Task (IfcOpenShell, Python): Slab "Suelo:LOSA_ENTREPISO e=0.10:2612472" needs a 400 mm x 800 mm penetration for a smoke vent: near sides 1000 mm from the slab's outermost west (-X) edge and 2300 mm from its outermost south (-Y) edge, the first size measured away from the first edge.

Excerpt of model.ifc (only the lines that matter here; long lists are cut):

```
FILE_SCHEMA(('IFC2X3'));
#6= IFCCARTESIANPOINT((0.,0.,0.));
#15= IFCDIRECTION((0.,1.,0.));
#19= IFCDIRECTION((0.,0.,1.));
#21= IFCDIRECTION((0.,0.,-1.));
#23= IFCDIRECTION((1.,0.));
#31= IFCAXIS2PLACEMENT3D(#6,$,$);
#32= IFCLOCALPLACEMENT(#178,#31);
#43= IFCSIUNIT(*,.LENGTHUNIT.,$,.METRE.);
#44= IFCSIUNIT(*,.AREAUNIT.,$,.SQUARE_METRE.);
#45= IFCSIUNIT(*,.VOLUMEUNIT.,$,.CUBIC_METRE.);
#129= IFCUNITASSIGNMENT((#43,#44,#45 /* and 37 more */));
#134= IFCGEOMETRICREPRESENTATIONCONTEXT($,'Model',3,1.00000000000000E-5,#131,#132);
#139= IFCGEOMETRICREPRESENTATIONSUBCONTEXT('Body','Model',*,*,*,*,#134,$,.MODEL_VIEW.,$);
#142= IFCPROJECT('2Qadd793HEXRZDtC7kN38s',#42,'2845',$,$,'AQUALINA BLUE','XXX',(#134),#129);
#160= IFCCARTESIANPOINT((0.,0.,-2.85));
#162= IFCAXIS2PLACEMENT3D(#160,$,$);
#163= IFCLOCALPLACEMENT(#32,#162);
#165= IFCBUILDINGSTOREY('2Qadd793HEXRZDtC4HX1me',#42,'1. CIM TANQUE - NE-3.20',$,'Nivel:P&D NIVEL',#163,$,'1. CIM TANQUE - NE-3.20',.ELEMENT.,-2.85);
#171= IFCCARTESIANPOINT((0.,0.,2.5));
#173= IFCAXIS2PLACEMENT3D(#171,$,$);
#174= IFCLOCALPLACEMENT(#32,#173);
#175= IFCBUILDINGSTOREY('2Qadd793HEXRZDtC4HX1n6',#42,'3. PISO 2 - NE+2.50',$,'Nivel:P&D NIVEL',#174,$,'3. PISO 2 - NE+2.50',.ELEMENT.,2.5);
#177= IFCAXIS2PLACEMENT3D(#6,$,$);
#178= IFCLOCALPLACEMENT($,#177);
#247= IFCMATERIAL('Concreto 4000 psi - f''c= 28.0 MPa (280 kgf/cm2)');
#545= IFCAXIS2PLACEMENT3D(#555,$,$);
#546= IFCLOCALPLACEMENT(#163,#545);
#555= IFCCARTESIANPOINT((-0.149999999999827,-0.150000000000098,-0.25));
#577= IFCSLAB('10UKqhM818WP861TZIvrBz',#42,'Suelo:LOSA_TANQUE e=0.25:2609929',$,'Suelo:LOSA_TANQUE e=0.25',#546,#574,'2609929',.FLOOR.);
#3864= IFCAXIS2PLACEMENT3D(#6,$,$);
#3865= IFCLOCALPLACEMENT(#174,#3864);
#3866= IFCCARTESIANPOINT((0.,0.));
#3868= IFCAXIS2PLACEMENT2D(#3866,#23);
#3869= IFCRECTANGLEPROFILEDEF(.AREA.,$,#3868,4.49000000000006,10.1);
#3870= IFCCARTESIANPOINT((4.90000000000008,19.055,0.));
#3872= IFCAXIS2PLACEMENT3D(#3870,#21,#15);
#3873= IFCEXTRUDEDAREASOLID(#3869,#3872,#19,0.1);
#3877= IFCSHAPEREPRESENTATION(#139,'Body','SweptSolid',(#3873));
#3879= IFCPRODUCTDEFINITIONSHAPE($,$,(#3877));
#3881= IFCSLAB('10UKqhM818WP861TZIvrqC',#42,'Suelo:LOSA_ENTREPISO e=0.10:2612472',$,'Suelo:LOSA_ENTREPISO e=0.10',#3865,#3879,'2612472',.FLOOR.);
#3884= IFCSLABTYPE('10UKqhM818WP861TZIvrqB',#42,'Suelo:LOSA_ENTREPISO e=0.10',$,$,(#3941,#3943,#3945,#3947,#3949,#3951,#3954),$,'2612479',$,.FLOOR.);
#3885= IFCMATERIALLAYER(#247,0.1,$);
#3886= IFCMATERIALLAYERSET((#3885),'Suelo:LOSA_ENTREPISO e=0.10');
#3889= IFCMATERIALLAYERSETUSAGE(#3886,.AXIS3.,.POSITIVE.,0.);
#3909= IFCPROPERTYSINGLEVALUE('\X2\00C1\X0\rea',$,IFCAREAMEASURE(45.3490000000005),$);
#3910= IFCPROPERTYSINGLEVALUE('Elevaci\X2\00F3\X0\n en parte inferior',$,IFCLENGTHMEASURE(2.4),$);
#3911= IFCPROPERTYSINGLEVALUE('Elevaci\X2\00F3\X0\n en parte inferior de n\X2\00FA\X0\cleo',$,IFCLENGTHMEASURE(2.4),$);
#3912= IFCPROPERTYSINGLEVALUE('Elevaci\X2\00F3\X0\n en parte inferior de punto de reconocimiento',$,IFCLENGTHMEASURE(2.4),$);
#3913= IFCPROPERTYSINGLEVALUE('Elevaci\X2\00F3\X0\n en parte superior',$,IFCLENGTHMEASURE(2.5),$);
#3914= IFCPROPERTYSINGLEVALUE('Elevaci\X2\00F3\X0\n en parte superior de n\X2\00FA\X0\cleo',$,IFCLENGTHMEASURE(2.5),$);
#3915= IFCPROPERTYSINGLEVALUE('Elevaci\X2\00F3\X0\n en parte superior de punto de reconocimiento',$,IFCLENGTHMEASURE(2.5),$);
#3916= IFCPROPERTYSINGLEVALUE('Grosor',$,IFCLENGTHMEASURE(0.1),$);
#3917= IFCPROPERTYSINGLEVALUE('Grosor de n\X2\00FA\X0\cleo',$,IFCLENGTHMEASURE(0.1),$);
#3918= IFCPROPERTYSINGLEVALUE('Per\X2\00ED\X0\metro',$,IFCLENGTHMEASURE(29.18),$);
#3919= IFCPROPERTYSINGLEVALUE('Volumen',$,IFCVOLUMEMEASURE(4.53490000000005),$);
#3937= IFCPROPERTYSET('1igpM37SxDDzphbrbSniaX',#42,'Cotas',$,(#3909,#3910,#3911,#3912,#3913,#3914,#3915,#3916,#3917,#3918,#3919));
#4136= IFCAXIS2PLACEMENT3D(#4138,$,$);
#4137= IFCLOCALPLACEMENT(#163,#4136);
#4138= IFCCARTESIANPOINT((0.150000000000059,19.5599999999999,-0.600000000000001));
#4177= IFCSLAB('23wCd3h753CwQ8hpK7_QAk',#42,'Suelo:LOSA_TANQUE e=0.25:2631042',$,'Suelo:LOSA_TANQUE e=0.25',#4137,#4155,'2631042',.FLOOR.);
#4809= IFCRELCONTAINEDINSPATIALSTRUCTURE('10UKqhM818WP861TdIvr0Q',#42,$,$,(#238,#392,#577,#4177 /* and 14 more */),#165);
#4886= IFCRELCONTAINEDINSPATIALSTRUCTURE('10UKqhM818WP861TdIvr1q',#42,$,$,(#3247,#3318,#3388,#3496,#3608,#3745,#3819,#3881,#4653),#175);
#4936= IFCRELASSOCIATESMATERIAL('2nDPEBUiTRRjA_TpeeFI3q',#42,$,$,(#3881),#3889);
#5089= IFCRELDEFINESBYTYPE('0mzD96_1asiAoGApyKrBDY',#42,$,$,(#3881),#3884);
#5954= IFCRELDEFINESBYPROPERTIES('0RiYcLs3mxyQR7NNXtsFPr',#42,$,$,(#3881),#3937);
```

```python
import numpy as np
import ifcopenshell
import ifcopenshell.api.feature
import ifcopenshell.api.geometry
import ifcopenshell.api.pset
import ifcopenshell.api.root
import ifcopenshell.geom
import ifcopenshell.util.element
import ifcopenshell.util.placement
import ifcopenshell.util.representation
import ifcopenshell.util.shape
import ifcopenshell.util.unit

model = ifcopenshell.open("model.ifc")
unit_scale = ifcopenshell.util.unit.calculate_unit_scale(model)
area_scale = ifcopenshell.util.unit.calculate_unit_scale(model, "AREAUNIT")
volume_scale = ifcopenshell.util.unit.calculate_unit_scale(model, "VOLUMEUNIT")
settings = ifcopenshell.geom.settings()


def volume(element):
    """Net volume in cubic metres, openings subtracted."""
    shape = ifcopenshell.geom.create_shape(settings, element)
    return ifcopenshell.util.shape.get_volume(shape.geometry)


slab = model.by_guid("10UKqhM818WP861TZIvrqC")
before = volume(slab)

# Extent in the slab's own axes, in metres. The edges named are its -X and -Y sides.
slab_shape = ifcopenshell.geom.create_shape(settings, slab)
vertices = ifcopenshell.util.shape.get_vertices(slab_shape.geometry)
x_min, y_min, bottom = vertices.min(axis=0)
top = vertices[:, 2].max()

opening = ifcopenshell.api.root.create_entity(model, ifc_class="IfcOpeningElement", name="Smoke vent opening")
context = ifcopenshell.util.representation.get_context(model, "Model", "Body", "MODEL_VIEW")
width, depth = 0.4, 0.8
outline = [(0.0, 0.0), (width, 0.0), (width, depth), (0.0, depth), (0.0, 0.0)]
# Overshoot both faces by 50 mm so the cut is clean.
shape = ifcopenshell.api.geometry.add_slab_representation(
    model, context=context, depth=top - bottom + 0.1, polyline=outline
)
ifcopenshell.api.geometry.assign_representation(model, product=opening, representation=shape)

matrix = ifcopenshell.util.placement.get_local_placement(slab.ObjectPlacement)
matrix[:, 3] = matrix @ np.append(np.array([x_min + 1, y_min + 2.3, bottom - 0.05]) / unit_scale, 1.0)
ifcopenshell.api.geometry.edit_object_placement(model, product=opening, matrix=matrix, is_si=False)
ifcopenshell.api.feature.add_feature(model, feature=opening, element=slab)

after = volume(slab)

# Update the slab's stored quantities.
pset = model.by_id(ifcopenshell.util.element.get_pset(slab, "Cotas", should_inherit=False)["id"])
ifcopenshell.api.pset.edit_pset(model, pset=pset, properties={
    "Área": model.create_entity("IfcAreaMeasure", after / (top - bottom) / area_scale),
    "Volumen": model.create_entity("IfcVolumeMeasure", after / volume_scale),
})

print(f"slab volume {before:.3f} -> {after:.3f} m3")

model.write("model_edited.ifc")
```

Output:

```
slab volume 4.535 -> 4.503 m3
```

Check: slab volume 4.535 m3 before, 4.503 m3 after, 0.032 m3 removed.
